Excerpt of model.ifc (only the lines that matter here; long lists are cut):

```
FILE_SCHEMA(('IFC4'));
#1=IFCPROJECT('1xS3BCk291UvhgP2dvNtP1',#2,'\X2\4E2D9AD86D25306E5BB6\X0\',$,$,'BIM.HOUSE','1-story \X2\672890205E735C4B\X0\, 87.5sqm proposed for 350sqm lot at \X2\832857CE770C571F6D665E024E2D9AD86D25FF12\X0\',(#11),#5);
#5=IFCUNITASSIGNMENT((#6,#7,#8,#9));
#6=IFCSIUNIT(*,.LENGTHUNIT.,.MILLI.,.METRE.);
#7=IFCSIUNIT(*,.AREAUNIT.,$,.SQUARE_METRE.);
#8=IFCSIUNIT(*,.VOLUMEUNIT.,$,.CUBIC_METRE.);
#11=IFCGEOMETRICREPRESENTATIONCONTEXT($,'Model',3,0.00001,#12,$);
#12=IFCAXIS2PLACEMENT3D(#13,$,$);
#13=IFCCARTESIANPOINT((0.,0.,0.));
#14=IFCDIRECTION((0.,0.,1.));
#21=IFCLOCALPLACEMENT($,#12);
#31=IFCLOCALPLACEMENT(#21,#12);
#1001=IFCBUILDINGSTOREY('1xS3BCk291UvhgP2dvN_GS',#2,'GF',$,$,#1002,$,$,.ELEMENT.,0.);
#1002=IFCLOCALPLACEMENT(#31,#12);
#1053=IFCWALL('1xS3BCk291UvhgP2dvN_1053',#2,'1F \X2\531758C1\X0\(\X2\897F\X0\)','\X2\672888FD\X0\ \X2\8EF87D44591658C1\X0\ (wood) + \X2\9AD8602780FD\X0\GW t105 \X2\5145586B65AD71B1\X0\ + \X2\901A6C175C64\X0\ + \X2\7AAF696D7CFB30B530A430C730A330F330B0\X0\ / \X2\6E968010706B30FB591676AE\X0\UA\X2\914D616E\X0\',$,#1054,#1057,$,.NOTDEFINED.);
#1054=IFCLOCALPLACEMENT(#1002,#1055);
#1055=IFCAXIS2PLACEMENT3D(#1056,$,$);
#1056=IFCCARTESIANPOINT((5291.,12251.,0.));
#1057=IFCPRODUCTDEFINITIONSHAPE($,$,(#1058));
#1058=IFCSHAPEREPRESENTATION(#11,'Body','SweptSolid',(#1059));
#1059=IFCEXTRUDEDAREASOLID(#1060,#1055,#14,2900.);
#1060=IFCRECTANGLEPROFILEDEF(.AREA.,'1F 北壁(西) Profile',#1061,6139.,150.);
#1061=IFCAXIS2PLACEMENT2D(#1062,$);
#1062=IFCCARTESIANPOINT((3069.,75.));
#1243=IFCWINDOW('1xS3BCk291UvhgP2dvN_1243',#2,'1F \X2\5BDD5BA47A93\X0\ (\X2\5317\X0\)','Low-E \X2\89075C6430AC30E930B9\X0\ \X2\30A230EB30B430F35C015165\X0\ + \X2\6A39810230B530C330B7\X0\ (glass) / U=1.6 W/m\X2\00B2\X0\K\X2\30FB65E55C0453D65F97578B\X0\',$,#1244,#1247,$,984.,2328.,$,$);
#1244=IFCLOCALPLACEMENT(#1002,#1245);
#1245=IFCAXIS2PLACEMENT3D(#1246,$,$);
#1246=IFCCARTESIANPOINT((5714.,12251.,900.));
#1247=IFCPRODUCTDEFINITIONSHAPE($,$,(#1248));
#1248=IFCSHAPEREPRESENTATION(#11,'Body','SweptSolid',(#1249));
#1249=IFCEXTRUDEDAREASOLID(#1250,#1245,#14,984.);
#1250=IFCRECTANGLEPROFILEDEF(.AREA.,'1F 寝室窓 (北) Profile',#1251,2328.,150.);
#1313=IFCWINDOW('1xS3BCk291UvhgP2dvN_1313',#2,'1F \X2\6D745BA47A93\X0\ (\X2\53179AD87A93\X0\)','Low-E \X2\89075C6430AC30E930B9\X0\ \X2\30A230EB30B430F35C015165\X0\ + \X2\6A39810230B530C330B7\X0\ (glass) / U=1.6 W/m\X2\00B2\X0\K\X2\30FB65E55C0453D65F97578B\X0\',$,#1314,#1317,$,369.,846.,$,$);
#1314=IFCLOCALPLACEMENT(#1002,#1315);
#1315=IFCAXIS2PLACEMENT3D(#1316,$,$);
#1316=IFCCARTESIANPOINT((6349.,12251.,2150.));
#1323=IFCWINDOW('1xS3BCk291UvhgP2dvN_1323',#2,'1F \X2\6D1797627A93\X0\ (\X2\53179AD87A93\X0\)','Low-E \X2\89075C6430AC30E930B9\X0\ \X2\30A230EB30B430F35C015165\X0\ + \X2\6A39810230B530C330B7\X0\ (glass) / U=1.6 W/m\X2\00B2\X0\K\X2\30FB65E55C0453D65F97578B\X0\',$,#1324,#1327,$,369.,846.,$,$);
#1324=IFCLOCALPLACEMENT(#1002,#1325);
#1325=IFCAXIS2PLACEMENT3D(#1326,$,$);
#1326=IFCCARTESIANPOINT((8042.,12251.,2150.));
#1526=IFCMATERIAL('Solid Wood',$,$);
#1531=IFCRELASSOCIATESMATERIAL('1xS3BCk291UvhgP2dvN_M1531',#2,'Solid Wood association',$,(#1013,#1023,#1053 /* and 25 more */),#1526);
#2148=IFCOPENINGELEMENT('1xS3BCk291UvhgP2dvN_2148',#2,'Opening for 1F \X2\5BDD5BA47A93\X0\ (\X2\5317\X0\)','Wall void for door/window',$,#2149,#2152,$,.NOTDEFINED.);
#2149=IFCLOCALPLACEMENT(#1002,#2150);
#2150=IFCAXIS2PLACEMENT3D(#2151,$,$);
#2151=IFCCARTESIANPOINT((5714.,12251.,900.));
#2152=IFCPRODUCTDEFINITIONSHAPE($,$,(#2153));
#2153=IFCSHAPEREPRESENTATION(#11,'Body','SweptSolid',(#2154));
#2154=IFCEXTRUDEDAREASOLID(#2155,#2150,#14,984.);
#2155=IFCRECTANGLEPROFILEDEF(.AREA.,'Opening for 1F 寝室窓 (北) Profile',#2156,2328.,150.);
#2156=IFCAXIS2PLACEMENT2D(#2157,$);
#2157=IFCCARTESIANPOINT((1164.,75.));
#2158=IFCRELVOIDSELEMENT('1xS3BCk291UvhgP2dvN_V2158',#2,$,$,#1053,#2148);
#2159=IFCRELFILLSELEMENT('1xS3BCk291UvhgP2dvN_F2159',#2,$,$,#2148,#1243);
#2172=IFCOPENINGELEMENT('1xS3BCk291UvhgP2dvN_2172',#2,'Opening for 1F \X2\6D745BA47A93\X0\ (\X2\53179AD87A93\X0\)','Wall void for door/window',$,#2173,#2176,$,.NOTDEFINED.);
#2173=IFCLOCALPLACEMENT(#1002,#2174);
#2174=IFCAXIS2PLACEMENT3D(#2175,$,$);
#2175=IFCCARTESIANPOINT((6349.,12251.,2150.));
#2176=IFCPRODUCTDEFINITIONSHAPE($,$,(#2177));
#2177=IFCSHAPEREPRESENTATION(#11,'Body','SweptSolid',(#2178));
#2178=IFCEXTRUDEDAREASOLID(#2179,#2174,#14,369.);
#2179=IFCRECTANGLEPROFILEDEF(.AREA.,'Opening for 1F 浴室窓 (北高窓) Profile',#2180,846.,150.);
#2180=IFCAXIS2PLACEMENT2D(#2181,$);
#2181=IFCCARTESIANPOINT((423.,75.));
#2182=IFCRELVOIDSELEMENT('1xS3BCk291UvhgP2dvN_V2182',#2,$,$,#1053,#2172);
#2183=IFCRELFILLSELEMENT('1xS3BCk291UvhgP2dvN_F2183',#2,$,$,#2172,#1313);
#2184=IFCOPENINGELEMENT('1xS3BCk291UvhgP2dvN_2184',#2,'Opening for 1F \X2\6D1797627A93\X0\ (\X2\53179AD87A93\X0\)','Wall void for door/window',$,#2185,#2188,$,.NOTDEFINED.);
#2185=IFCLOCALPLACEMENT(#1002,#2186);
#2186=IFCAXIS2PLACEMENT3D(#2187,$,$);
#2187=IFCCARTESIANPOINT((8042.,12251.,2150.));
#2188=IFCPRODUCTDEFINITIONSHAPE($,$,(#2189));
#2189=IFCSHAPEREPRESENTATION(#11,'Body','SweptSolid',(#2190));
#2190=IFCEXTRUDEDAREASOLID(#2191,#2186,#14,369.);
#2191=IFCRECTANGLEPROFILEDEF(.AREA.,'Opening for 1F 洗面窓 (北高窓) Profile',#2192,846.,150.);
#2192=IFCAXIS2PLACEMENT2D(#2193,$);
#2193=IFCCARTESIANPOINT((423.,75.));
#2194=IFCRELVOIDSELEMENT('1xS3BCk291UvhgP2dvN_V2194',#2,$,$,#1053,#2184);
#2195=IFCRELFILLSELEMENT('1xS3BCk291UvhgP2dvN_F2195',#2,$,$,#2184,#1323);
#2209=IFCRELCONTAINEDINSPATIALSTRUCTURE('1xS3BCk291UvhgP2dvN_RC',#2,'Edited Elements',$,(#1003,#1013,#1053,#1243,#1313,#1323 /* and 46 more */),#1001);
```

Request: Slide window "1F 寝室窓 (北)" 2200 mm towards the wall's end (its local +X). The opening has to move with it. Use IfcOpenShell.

```python
import ifcopenshell
import ifcopenshell.api.geometry
import ifcopenshell.util.placement
import ifcopenshell.util.unit

model = ifcopenshell.open("model.ifc")
unit_scale = ifcopenshell.util.unit.calculate_unit_scale(model)

window = model.by_guid("1xS3BCk291UvhgP2dvN_1243")
opening = window.FillsVoids[0].RelatingOpeningElement
wall = opening.VoidsElements[0].RelatingBuildingElement

wall_matrix = ifcopenshell.util.placement.get_local_placement(wall.ObjectPlacement)
shift = wall_matrix[:3, 0] * 2.2 / unit_scale
before = ifcopenshell.util.placement.get_local_placement(window.ObjectPlacement)[:3, 3].copy()

# The window is not placed relative to its opening, so move both.
for product in (opening, window):
    matrix = ifcopenshell.util.placement.get_local_placement(product.ObjectPlacement)
    matrix[:3, 3] += shift
    ifcopenshell.api.geometry.edit_object_placement(model, product=product, matrix=matrix, is_si=False)

after = ifcopenshell.util.placement.get_local_placement(window.ObjectPlacement)[:3, 3]
print("window moved by", (after - before).round(3) + 0.0)

model.write("model_edited.ifc")
```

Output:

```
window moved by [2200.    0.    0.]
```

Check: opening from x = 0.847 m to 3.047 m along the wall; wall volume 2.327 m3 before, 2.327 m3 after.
